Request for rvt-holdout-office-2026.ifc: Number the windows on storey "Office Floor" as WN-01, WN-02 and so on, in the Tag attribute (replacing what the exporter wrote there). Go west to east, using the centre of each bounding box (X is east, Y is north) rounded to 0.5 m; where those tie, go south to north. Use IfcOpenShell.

First a look at what the model holds.

```python
import ifcopenshell
import ifcopenshell.util.element
import ifcopenshell.util.placement

model = ifcopenshell.open("rvt-holdout-office-2026.ifc")
print(model.schema)
storey = next(s for s in model.by_type("IfcBuildingStorey") if s.Name == "Office Floor")
windows = [e for e in ifcopenshell.util.element.get_decomposition(storey) if e.is_a("IfcWindow")]
for e in sorted(windows, key=lambda e: e.id()):
    origin = ifcopenshell.util.placement.get_local_placement(e.ObjectPlacement)[:3, 3]
    print(e.id(), e.Tag, e.Name, origin.round(2) + 0.0, sep=" | ")
```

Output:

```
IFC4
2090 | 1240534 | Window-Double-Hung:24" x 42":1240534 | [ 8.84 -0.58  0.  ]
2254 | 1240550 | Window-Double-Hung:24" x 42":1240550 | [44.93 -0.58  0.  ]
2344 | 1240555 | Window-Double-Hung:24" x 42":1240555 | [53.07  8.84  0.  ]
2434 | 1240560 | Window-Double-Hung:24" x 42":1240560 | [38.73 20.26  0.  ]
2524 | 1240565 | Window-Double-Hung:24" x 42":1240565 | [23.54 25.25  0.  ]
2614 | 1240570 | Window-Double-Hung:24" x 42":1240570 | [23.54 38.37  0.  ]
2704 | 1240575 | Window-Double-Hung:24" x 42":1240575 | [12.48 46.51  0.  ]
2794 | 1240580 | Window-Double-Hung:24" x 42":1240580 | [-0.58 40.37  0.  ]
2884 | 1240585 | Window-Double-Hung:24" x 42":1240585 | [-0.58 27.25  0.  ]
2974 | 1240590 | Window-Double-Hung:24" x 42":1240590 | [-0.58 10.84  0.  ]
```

```python
import ifcopenshell
import ifcopenshell.geom
import ifcopenshell.util.element
import ifcopenshell.util.shape

model = ifcopenshell.open("rvt-holdout-office-2026.ifc")
settings = ifcopenshell.geom.settings()
settings.set("use-world-coords", True)


def centre(element):
    shape = ifcopenshell.geom.create_shape(settings, element)
    return ifcopenshell.util.shape.get_bbox_centroid(shape.geometry)


storey = next(s for s in model.by_type("IfcBuildingStorey") if s.Name == "Office Floor")
windows = [e for e in ifcopenshell.util.element.get_decomposition(storey) if e.is_a("IfcWindow")]

# Insertion points can sit at a corner or the storey origin, so sort by the geometry (in metres).
centres = {e: centre(e) for e in windows}
windows.sort(key=lambda e: (round(centres[e][0] / 0.5), centres[e][1]))

for i, e in enumerate(windows, start=1):
    number = f"WN-{i:02d}"
    e.Tag = number
    print(e.id(), number)

model.write("rvt-holdout-office-2026-out.ifc")
```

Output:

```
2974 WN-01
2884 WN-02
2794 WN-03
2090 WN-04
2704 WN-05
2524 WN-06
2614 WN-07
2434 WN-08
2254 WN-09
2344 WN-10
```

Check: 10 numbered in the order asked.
